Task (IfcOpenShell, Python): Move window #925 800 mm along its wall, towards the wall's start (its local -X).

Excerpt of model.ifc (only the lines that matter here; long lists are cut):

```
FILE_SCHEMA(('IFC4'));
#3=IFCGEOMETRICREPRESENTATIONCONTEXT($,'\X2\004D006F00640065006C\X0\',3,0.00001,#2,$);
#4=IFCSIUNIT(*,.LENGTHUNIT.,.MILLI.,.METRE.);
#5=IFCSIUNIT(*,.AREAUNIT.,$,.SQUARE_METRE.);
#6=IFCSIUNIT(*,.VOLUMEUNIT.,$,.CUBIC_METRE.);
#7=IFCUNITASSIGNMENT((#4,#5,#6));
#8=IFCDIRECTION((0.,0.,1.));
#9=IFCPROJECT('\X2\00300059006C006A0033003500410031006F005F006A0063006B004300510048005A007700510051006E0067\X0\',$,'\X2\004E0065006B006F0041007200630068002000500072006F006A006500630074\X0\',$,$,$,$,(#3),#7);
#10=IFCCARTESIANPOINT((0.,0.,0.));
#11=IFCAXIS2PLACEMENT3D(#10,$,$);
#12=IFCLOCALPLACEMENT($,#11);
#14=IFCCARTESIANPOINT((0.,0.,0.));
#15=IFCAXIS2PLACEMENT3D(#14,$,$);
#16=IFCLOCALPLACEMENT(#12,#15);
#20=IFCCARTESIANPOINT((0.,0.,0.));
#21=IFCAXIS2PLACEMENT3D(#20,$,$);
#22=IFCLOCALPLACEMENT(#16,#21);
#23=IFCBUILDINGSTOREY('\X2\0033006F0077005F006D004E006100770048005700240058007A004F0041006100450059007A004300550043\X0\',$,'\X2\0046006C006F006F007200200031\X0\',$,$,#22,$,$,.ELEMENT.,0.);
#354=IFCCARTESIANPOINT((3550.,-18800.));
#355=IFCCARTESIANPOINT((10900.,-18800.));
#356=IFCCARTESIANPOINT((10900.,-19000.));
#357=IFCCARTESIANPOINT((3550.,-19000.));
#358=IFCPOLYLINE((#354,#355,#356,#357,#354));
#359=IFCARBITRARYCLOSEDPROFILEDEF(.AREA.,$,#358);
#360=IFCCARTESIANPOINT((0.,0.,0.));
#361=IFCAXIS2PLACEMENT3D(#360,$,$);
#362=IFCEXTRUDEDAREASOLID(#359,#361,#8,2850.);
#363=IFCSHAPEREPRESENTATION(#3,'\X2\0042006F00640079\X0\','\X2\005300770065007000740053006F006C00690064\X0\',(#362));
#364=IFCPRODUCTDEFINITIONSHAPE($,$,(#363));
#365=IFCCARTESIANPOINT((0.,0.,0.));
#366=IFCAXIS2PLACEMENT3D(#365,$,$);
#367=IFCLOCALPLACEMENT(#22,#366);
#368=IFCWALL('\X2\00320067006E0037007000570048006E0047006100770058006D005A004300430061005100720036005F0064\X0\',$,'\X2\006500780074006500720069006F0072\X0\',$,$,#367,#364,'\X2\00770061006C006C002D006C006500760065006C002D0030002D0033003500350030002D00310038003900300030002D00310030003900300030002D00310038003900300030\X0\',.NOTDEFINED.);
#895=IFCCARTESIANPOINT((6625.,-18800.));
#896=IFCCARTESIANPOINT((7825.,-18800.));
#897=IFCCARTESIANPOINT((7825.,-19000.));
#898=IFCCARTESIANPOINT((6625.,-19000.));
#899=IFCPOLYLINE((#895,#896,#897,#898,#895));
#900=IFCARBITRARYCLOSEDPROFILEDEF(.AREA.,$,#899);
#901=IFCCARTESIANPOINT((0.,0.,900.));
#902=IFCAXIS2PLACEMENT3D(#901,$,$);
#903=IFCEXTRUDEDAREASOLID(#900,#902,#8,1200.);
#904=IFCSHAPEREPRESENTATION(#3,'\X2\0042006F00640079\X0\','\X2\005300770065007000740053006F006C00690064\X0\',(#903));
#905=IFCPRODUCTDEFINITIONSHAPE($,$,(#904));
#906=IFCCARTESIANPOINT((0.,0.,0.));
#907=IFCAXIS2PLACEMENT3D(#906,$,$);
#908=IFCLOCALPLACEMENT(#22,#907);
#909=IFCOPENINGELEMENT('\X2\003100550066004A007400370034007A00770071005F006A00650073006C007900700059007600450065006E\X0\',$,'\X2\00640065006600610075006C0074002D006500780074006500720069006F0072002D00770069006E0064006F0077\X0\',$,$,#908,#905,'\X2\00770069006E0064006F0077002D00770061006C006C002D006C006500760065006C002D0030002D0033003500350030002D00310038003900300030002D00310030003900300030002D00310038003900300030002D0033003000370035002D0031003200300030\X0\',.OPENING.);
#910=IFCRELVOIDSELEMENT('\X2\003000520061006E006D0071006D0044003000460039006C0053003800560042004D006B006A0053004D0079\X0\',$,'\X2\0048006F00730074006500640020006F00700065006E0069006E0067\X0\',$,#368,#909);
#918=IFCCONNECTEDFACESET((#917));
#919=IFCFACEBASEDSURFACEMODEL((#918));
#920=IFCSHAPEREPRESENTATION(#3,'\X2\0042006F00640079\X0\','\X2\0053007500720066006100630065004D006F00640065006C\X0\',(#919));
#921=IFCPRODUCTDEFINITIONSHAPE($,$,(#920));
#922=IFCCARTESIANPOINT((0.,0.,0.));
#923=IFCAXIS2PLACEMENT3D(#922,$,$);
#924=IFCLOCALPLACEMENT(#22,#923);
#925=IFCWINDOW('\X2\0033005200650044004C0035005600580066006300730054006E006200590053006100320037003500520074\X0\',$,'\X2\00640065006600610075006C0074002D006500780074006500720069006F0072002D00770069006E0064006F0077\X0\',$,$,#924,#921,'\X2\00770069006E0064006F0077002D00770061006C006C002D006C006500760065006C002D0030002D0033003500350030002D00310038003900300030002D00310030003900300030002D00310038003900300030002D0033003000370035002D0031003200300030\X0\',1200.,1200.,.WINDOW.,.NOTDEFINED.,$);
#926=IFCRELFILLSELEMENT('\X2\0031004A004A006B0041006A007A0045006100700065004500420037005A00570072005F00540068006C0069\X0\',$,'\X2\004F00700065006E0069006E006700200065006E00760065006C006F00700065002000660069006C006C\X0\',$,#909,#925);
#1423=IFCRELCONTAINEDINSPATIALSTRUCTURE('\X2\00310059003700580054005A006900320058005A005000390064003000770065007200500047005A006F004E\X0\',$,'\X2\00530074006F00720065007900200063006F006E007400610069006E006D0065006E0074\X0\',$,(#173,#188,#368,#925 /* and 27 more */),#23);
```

```python
import ifcopenshell
import ifcopenshell.api.geometry
import ifcopenshell.util.placement

model = ifcopenshell.open("model.ifc")

window = model.by_guid("3ReDL5VXfcsTnbYSa275Rt")
opening = window.FillsVoids[0].RelatingOpeningElement
wall = opening.VoidsElements[0].RelatingBuildingElement

wall_matrix = ifcopenshell.util.placement.get_local_placement(wall.ObjectPlacement)
shift = wall_matrix[:3, 0] * -800.0
before = ifcopenshell.util.placement.get_local_placement(window.ObjectPlacement)[:3, 3].copy()

# The window is not placed relative to its opening, so move both.
for product in (opening, window):
    matrix = ifcopenshell.util.placement.get_local_placement(product.ObjectPlacement)
    matrix[:3, 3] += shift
    ifcopenshell.api.geometry.edit_object_placement(model, product=product, matrix=matrix, is_si=False)

after = ifcopenshell.util.placement.get_local_placement(window.ObjectPlacement)[:3, 3]
print("window moved by", (after - before).round(3) + 0.0)

model.write("model_updated.ifc")
```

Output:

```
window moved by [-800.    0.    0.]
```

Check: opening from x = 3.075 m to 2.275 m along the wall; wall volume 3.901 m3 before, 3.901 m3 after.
